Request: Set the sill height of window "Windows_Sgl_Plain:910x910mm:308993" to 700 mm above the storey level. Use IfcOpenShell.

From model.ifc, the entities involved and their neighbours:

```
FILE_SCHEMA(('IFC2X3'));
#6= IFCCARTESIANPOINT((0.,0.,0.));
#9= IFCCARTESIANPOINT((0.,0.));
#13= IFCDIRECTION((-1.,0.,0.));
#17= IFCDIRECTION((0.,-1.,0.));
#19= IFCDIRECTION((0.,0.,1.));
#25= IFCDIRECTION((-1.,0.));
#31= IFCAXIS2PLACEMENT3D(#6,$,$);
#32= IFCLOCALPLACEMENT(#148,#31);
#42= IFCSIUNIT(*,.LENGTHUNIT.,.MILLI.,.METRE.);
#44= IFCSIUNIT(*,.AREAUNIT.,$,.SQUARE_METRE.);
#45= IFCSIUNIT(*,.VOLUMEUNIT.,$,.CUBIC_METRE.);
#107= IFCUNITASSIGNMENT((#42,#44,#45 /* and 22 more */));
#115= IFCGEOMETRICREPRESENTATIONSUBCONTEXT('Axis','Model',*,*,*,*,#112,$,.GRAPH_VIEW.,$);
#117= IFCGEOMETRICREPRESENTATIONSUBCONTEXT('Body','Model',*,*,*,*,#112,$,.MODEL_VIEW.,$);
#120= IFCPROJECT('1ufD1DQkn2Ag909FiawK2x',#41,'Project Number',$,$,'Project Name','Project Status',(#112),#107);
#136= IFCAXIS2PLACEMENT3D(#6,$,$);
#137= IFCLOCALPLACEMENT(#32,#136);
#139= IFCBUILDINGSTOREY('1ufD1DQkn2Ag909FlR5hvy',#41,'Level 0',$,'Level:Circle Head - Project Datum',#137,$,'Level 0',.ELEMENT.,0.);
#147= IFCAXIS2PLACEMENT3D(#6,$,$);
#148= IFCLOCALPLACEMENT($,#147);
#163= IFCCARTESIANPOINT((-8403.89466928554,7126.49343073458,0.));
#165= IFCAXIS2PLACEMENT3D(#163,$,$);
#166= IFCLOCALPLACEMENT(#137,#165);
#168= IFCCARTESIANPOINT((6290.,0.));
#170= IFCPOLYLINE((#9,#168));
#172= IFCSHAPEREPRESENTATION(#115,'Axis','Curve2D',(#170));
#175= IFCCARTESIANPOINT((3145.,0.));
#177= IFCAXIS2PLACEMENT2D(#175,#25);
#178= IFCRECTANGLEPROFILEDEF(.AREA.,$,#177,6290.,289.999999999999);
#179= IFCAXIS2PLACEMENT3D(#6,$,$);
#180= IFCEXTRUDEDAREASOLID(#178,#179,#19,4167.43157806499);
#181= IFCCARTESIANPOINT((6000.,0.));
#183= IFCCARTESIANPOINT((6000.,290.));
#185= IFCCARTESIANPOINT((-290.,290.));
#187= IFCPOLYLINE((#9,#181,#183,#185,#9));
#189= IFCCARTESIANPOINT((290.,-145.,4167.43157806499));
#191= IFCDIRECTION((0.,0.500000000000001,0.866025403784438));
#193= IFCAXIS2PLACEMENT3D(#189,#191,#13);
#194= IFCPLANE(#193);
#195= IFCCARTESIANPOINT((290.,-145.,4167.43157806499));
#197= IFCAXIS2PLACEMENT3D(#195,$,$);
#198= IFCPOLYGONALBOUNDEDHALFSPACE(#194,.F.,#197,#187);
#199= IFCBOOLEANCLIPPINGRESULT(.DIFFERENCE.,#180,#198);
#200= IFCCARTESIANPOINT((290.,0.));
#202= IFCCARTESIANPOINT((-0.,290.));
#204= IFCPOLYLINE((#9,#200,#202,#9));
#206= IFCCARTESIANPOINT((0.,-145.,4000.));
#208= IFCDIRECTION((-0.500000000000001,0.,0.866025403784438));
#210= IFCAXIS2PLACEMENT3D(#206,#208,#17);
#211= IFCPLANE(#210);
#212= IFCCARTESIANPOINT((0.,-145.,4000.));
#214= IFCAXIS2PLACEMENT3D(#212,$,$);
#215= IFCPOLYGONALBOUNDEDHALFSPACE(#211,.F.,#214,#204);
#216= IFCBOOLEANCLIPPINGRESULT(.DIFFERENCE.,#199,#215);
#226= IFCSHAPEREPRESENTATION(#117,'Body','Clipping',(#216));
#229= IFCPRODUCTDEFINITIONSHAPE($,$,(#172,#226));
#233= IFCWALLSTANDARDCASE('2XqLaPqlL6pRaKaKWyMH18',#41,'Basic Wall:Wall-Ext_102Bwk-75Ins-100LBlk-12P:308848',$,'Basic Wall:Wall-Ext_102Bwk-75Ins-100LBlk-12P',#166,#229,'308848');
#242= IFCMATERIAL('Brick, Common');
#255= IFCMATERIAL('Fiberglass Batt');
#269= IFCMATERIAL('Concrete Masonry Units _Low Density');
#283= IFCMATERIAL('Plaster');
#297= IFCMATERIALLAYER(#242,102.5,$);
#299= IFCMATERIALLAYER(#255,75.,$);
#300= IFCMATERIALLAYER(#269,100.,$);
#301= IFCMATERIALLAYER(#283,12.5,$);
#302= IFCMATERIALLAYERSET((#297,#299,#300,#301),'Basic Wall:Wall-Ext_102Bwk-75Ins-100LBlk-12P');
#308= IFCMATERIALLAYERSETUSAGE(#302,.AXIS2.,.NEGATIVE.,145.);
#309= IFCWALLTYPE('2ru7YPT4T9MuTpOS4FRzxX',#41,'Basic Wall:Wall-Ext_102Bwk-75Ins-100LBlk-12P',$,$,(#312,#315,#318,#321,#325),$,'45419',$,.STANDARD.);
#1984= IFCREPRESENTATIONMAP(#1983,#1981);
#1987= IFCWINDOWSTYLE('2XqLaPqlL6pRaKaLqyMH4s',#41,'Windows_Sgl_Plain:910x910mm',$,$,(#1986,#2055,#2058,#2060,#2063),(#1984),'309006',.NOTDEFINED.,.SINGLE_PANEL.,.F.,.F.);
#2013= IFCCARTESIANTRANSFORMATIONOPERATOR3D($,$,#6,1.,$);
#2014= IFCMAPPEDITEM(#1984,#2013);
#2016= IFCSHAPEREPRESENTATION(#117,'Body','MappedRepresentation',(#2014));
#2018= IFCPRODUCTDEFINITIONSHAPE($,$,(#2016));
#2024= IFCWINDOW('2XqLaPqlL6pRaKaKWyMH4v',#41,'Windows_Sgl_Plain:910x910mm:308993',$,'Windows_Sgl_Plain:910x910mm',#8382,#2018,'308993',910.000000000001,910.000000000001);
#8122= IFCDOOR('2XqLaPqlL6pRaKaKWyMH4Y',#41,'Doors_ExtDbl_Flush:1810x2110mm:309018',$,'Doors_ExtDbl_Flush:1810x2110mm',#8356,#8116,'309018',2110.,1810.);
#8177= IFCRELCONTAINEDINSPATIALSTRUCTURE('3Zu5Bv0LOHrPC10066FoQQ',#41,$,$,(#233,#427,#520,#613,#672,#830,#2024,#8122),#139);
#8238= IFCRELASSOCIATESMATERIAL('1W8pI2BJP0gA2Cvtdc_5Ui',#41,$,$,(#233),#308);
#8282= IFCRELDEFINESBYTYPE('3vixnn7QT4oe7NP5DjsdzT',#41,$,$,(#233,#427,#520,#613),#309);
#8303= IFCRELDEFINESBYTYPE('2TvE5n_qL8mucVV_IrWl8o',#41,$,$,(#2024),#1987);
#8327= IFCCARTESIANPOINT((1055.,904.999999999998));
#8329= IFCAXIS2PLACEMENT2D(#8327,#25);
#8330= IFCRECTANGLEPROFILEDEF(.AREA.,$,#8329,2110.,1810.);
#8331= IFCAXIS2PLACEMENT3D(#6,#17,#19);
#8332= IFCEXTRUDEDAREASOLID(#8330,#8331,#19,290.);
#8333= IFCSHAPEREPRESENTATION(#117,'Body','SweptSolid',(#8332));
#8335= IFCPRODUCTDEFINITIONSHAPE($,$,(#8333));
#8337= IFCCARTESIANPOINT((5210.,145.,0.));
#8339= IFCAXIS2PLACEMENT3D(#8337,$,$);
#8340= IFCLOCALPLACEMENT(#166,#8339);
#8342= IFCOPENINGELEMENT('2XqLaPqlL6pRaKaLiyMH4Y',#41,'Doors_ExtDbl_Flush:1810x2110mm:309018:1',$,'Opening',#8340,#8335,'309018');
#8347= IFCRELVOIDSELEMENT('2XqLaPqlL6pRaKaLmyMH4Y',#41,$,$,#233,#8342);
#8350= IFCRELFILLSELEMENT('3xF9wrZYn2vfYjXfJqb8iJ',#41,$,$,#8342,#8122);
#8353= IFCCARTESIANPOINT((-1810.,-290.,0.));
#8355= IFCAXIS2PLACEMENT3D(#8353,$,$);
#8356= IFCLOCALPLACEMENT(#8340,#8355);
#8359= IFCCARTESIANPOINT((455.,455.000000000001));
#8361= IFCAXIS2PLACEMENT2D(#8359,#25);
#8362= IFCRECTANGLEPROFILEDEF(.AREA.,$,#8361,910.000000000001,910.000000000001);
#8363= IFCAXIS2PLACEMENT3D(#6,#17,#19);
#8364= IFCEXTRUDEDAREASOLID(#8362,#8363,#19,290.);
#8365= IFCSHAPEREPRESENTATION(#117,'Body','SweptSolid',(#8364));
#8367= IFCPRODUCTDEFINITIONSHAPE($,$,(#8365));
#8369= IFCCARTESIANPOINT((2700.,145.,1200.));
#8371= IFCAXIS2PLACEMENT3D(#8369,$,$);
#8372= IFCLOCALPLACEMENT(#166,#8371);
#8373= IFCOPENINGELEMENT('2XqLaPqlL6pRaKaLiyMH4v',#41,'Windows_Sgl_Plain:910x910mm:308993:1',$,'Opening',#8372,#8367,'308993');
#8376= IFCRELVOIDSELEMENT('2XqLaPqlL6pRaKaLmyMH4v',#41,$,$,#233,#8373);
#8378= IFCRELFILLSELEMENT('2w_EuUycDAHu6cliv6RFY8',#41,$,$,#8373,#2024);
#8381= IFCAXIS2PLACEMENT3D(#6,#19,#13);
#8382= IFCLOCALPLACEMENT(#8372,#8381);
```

```python
import numpy as np
import ifcopenshell
import ifcopenshell.api.geometry
import ifcopenshell.geom
import ifcopenshell.util.element
import ifcopenshell.util.placement
import ifcopenshell.util.shape
import ifcopenshell.util.unit

model = ifcopenshell.open("model.ifc")
unit_scale = ifcopenshell.util.unit.calculate_unit_scale(model)

window = model.by_guid("2XqLaPqlL6pRaKaKWyMH4v")
opening = window.FillsVoids[0].RelatingOpeningElement
storey = ifcopenshell.util.element.get_container(window, ifc_class="IfcBuildingStorey")
level = ifcopenshell.util.placement.get_local_placement(storey.ObjectPlacement)[2, 3]

# The opening's origin need not be at the sill, so measure its lowest point.
shape = ifcopenshell.geom.create_shape(ifcopenshell.geom.settings(), opening)
bottom = ifcopenshell.util.shape.get_shape_bottom_elevation(shape, shape.geometry) / unit_scale
dz = level + 0.7 / unit_scale - bottom

shift = np.array([0.0, 0.0, dz])
# The window is placed relative to its opening, so it follows when the opening moves.
matrix = ifcopenshell.util.placement.get_local_placement(opening.ObjectPlacement)
matrix[:3, 3] += shift
ifcopenshell.api.geometry.edit_object_placement(
    model, product=opening, matrix=matrix, is_si=False, should_transform_children=True
)

print(f"moved by {dz * unit_scale:+.3f} m")

model.write("model_edited.ifc")
```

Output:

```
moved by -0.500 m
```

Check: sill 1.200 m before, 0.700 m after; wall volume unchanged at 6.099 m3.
